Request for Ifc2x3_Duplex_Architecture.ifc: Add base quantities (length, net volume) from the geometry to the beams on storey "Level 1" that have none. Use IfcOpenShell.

First a look at what the model holds.

```python
import ifcopenshell
import ifcopenshell.util.element
import ifcopenshell.util.unit

model = ifcopenshell.open("Ifc2x3_Duplex_Architecture.ifc")
print(model.schema)
for unit_type in ("LENGTHUNIT", "AREAUNIT", "VOLUMEUNIT"):
    print(unit_type, ifcopenshell.util.unit.calculate_unit_scale(model, unit_type))
storey = next(s for s in model.by_type("IfcBuildingStorey") if s.Name == "Level 1")
beams = [e for e in ifcopenshell.util.element.get_decomposition(storey) if e.is_a("IfcBeam")]
for e in sorted(beams, key=lambda e: e.id()):
    print(e.id(), e.is_a(), e.Name, list(ifcopenshell.util.element.get_psets(e, qtos_only=True)), sep=" | ")
```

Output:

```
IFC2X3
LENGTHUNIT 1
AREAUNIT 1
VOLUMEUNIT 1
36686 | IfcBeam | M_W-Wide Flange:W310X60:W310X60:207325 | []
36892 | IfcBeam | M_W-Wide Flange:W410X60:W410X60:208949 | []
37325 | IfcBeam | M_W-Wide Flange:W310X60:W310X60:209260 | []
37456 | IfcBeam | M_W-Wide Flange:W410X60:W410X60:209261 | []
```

```python
import ifcopenshell
import ifcopenshell.api.pset
import ifcopenshell.geom
import ifcopenshell.util.element
import ifcopenshell.util.shape
import ifcopenshell.util.unit

model = ifcopenshell.open("Ifc2x3_Duplex_Architecture.ifc")
unit_scale = ifcopenshell.util.unit.calculate_unit_scale(model)
volume_scale = ifcopenshell.util.unit.calculate_unit_scale(model, "VOLUMEUNIT")
settings = ifcopenshell.geom.settings()

storey = next(s for s in model.by_type("IfcBuildingStorey") if s.Name == "Level 1")
beams = [e for e in ifcopenshell.util.element.get_decomposition(storey) if e.is_a("IfcBeam")]

for e in sorted(beams, key=lambda e: e.id()):
    if ifcopenshell.util.element.get_psets(e, qtos_only=True, should_inherit=False):
        continue
    # Geometry comes back in metres, in the element's own axes.
    shape = ifcopenshell.geom.create_shape(settings, e)
    values = {
        "Length": ifcopenshell.util.shape.get_max_xyz(shape.geometry) / unit_scale,
        "NetVolume": ifcopenshell.util.shape.get_volume(shape.geometry) / volume_scale,
    }
    qto = ifcopenshell.api.pset.add_qto(model, product=e, name="BaseQuantities")
    ifcopenshell.api.pset.edit_qto(model, qto=qto, properties=values)
    print(e.id(), {k: round(v, 3) for k, v in values.items()})

model.write("Ifc2x3_Duplex_Architecture-out.ifc")
```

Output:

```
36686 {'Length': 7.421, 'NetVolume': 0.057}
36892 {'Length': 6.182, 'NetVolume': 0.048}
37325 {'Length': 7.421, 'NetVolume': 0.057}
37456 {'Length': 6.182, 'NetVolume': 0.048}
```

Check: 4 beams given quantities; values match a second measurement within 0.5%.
